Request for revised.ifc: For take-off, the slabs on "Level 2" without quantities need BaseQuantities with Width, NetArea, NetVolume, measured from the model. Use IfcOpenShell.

First a look at what the model holds.

```python
import ifcopenshell
import ifcopenshell.util.element
import ifcopenshell.util.unit

model = ifcopenshell.open("revised.ifc")
print(model.schema)
for unit_type in ("LENGTHUNIT", "AREAUNIT", "VOLUMEUNIT"):
    print(unit_type, ifcopenshell.util.unit.calculate_unit_scale(model, unit_type))
storey = next(s for s in model.by_type("IfcBuildingStorey") if s.Name == "Level 2")
slabs = [e for e in ifcopenshell.util.element.get_decomposition(storey) if e.is_a("IfcSlab")]
for e in sorted(slabs, key=lambda e: e.id()):
    print(e.id(), e.is_a(), e.Name, list(ifcopenshell.util.element.get_psets(e, qtos_only=True)), sep=" | ")
```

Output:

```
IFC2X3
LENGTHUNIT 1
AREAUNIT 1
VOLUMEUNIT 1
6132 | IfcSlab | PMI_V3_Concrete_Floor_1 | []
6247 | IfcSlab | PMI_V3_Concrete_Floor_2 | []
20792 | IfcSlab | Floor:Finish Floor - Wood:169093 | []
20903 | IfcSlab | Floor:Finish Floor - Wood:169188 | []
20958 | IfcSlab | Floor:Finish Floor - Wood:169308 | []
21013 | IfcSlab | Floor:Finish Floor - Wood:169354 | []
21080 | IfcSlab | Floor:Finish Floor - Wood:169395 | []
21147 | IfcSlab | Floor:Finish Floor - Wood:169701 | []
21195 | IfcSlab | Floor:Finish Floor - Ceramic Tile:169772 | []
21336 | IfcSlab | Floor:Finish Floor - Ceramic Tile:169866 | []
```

```python
import ifcopenshell
import ifcopenshell.api.pset
import ifcopenshell.geom
import ifcopenshell.util.element
import ifcopenshell.util.shape
import ifcopenshell.util.unit

model = ifcopenshell.open("revised.ifc")
unit_scale = ifcopenshell.util.unit.calculate_unit_scale(model)
area_scale = ifcopenshell.util.unit.calculate_unit_scale(model, "AREAUNIT")
volume_scale = ifcopenshell.util.unit.calculate_unit_scale(model, "VOLUMEUNIT")
settings = ifcopenshell.geom.settings()

storey = next(s for s in model.by_type("IfcBuildingStorey") if s.Name == "Level 2")
slabs = [e for e in ifcopenshell.util.element.get_decomposition(storey) if e.is_a("IfcSlab")]

for e in sorted(slabs, key=lambda e: e.id()):
    if ifcopenshell.util.element.get_psets(e, qtos_only=True, should_inherit=False):
        continue
    # Geometry comes back in metres, in the element's own axes.
    shape = ifcopenshell.geom.create_shape(settings, e)
    values = {
        "Width": ifcopenshell.util.shape.get_z(shape.geometry) / unit_scale,
        "NetArea": ifcopenshell.util.shape.get_footprint_area(shape.geometry) / area_scale,
        "NetVolume": ifcopenshell.util.shape.get_volume(shape.geometry) / volume_scale,
    }
    qto = ifcopenshell.api.pset.add_qto(model, product=e, name="BaseQuantities")
    ifcopenshell.api.pset.edit_qto(model, qto=qto, properties=values)
    print(e.id(), {k: round(v, 3) for k, v in values.items()})

model.write("revised_rev.ifc")
```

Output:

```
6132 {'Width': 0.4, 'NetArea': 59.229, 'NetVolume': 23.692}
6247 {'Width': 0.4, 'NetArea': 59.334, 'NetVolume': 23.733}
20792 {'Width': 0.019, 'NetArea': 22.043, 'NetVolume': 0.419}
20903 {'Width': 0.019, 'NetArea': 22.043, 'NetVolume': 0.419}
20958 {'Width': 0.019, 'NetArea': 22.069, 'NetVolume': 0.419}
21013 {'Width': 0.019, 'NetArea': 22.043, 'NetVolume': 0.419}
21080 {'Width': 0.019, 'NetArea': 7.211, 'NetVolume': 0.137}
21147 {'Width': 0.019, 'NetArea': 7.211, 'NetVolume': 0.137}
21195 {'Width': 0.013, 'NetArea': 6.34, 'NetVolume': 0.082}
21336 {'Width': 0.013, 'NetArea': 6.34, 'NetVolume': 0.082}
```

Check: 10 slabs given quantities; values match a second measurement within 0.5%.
